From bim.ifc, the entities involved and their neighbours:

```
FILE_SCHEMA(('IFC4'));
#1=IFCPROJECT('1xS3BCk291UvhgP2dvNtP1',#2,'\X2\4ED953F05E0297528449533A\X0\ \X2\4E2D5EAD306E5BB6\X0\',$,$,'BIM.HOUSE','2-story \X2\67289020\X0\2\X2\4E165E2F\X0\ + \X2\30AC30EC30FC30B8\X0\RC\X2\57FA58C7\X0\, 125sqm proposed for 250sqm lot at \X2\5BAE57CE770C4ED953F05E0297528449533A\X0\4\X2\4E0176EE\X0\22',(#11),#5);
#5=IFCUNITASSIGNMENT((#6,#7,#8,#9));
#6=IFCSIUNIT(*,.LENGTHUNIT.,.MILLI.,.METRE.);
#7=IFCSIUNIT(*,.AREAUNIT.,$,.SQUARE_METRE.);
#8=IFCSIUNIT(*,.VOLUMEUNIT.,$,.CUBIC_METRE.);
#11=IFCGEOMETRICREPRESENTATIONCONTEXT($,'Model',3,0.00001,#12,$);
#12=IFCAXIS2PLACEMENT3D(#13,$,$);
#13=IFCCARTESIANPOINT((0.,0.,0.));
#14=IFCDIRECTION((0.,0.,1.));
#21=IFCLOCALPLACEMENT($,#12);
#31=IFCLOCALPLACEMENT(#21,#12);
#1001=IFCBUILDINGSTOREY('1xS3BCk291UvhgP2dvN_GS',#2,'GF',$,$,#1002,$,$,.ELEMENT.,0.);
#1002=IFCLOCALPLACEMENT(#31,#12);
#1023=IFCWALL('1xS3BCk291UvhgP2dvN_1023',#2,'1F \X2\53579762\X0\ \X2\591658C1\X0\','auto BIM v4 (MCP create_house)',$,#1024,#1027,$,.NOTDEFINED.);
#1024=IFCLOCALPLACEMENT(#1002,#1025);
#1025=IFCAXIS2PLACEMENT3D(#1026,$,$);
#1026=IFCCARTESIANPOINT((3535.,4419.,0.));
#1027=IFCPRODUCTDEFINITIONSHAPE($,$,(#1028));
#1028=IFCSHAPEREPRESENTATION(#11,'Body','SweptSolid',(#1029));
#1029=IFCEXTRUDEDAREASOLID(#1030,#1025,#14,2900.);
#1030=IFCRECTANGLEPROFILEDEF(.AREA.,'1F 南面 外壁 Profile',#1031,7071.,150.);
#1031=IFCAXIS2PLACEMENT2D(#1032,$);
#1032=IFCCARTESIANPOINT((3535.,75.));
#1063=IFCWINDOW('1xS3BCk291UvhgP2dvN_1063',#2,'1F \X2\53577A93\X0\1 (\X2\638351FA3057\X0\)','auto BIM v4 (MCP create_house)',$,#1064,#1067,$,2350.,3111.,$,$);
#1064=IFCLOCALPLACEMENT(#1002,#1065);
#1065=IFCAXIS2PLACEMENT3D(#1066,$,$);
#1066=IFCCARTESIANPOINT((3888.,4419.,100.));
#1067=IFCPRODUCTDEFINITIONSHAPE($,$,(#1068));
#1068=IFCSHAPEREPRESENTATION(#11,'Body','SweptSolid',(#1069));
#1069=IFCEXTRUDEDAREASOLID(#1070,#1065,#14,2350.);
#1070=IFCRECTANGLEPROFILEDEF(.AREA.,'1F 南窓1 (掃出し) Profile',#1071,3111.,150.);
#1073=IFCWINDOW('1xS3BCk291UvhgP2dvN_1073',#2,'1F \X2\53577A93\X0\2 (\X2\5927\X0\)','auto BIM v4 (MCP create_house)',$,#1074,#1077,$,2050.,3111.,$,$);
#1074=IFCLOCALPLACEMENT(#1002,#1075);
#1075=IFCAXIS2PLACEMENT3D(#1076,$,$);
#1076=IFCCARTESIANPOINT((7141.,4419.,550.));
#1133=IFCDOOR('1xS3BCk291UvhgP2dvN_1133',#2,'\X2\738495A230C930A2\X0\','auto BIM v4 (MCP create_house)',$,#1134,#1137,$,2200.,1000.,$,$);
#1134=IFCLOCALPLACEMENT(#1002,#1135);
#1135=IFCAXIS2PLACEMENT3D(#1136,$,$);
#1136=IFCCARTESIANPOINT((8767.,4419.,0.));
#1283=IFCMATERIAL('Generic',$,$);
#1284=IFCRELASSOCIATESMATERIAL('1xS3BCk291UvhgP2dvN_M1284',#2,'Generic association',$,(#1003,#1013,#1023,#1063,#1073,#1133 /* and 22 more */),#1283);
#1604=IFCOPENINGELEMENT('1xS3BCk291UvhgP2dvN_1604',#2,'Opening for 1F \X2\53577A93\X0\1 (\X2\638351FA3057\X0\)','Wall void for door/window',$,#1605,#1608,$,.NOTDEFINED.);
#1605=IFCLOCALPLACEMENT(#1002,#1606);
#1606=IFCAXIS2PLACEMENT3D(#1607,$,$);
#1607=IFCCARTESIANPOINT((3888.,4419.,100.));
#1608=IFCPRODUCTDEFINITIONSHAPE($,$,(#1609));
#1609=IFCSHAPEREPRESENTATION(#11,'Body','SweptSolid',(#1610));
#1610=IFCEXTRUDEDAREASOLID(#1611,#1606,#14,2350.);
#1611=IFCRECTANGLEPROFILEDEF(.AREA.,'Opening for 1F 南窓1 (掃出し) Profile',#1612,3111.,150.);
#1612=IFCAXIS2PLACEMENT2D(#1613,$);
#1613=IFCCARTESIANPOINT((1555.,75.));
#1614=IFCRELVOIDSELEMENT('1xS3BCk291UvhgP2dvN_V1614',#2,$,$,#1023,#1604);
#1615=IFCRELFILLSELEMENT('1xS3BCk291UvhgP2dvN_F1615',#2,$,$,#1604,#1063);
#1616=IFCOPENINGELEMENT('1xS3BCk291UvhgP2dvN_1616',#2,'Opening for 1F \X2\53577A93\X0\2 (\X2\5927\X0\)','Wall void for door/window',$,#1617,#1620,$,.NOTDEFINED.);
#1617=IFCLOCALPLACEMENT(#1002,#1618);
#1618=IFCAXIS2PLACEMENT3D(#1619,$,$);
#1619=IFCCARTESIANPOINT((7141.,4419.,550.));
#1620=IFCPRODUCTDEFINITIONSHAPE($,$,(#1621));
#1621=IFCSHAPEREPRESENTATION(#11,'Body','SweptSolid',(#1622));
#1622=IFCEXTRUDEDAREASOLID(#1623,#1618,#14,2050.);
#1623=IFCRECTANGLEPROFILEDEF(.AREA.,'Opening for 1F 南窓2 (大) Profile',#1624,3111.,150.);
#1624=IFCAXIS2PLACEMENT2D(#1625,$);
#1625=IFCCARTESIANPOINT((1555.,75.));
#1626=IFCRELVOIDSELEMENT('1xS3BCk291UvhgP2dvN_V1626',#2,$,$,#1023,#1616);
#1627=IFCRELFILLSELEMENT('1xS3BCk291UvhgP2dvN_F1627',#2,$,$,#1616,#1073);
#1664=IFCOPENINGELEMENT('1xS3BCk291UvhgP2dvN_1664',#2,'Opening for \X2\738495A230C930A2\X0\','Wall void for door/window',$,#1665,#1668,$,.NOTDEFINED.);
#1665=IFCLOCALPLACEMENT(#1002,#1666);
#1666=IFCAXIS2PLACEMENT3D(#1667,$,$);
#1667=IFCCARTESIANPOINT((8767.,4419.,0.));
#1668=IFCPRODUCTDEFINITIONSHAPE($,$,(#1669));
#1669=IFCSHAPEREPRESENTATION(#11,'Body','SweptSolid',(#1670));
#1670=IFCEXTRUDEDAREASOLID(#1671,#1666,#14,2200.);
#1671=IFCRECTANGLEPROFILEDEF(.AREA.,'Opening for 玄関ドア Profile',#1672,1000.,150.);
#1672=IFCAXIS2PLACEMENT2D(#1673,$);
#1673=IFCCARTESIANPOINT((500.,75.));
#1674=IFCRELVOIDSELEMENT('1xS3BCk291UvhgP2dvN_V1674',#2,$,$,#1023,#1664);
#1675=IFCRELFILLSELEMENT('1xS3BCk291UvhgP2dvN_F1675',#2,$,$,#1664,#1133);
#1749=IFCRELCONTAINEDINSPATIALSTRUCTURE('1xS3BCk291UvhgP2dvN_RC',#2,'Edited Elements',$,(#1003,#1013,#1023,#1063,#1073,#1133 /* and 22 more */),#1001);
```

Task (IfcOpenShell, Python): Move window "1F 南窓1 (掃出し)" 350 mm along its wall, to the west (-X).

```python
import ifcopenshell
import ifcopenshell.api.geometry
import ifcopenshell.util.placement
import ifcopenshell.util.unit

model = ifcopenshell.open("bim.ifc")
unit_scale = ifcopenshell.util.unit.calculate_unit_scale(model)

window = model.by_guid("1xS3BCk291UvhgP2dvN_1063")
opening = window.FillsVoids[0].RelatingOpeningElement
wall = opening.VoidsElements[0].RelatingBuildingElement

wall_matrix = ifcopenshell.util.placement.get_local_placement(wall.ObjectPlacement)
shift = wall_matrix[:3, 0] * -0.35 / unit_scale
before = ifcopenshell.util.placement.get_local_placement(window.ObjectPlacement)[:3, 3].copy()

# The window is not placed relative to its opening, so move both.
for product in (opening, window):
    matrix = ifcopenshell.util.placement.get_local_placement(product.ObjectPlacement)
    matrix[:3, 3] += shift
    ifcopenshell.api.geometry.edit_object_placement(model, product=product, matrix=matrix, is_si=False)

after = ifcopenshell.util.placement.get_local_placement(window.ObjectPlacement)[:3, 3]
print("window moved by", (after - before).round(3) + 0.0)

model.write("bim_v2.ifc")
```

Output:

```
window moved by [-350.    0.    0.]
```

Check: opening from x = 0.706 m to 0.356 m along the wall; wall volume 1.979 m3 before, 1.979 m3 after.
